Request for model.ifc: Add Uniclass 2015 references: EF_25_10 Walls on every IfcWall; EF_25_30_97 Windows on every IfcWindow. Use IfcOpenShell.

First a look at what the model holds.

```python
import ifcopenshell

model = ifcopenshell.open("model.ifc")
print(model.schema)
print("classifications:", [c.Name for c in model.by_type("IfcClassification")])
for ifc_class in ("IfcDoor", "IfcRoof", "IfcStair", "IfcWall", "IfcWindow"):
    print(ifc_class, len(model.by_type(ifc_class)))
```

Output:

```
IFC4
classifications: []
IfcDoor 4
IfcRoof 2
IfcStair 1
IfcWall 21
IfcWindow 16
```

```python
import ifcopenshell
import ifcopenshell.api.classification

model = ifcopenshell.open("model.ifc")

system = ifcopenshell.api.classification.add_classification(model, classification="Uniclass 2015")

codes = {
    "IfcWall": ("EF_25_10", "Walls"),
    "IfcWindow": ("EF_25_30_97", "Windows"),
}
for ifc_class, (code, name) in codes.items():
    products = model.by_type(ifc_class)
    ifcopenshell.api.classification.add_reference(
        model, products=products, classification=system, identification=code, name=name
    )
    print(code, len(products))

model.write("model_rev.ifc")
```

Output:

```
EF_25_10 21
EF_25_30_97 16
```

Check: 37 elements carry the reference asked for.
